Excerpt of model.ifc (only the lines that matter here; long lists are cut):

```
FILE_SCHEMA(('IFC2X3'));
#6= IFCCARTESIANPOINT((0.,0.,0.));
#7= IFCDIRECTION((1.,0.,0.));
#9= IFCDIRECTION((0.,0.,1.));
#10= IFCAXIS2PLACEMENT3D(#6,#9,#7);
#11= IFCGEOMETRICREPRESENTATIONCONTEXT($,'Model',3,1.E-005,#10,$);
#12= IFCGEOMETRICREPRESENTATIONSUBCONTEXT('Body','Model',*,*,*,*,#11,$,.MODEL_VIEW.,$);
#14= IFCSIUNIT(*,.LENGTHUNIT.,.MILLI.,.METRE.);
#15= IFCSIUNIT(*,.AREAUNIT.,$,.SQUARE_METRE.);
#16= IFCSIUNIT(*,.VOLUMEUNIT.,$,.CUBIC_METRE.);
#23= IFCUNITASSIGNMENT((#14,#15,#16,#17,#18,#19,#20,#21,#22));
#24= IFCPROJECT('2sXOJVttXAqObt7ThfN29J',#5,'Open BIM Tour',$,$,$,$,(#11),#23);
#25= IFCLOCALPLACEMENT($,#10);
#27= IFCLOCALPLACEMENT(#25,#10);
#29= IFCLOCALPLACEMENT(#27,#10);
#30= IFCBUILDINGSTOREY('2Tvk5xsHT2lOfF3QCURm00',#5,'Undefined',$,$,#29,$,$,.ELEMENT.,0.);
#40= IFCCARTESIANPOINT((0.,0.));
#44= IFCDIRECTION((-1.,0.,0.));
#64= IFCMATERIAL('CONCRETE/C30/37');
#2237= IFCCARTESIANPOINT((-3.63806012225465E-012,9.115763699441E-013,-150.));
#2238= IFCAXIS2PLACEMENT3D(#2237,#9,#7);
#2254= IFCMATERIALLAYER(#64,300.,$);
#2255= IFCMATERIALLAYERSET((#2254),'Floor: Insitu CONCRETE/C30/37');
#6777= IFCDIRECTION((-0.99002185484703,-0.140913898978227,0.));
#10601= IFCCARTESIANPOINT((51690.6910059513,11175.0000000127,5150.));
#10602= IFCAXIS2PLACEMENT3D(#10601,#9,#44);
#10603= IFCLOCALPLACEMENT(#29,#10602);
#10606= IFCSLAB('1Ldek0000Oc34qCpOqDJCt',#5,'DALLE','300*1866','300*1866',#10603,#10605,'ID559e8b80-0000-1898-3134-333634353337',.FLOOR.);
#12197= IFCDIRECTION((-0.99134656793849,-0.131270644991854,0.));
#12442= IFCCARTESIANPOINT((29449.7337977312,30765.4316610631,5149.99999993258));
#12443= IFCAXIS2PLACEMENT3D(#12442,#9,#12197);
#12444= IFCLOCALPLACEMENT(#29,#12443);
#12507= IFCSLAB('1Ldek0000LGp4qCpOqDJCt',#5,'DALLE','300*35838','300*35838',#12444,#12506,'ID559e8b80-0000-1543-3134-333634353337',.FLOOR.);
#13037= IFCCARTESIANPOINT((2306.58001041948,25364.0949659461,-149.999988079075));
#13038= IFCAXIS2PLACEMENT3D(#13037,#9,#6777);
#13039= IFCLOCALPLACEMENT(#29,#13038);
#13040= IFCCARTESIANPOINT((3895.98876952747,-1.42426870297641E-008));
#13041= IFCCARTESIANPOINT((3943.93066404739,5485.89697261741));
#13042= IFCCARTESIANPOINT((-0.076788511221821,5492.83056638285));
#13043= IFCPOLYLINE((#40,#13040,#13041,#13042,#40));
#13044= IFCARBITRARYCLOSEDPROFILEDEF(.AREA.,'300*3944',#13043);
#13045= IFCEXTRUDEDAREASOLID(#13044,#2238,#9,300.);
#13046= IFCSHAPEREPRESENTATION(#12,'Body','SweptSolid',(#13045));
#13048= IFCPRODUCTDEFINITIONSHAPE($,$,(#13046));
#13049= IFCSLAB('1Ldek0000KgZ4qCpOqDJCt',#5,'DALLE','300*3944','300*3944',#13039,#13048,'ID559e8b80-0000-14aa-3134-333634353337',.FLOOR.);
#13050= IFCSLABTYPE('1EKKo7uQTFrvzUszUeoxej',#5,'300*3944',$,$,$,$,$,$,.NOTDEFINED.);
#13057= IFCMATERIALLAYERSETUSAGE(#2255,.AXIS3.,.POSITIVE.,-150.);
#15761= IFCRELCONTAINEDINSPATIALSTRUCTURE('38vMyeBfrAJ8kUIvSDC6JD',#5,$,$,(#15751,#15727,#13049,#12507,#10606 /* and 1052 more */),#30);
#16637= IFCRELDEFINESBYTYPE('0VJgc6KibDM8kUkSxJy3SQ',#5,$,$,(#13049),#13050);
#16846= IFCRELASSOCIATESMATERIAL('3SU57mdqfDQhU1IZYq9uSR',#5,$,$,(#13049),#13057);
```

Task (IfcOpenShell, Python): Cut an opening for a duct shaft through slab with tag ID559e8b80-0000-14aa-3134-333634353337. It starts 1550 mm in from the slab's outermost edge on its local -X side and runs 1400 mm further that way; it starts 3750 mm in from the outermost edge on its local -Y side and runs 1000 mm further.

```python
import numpy as np
import ifcopenshell
import ifcopenshell.api.feature
import ifcopenshell.api.geometry
import ifcopenshell.api.root
import ifcopenshell.geom
import ifcopenshell.util.placement
import ifcopenshell.util.representation
import ifcopenshell.util.shape
import ifcopenshell.util.unit

model = ifcopenshell.open("model.ifc")
unit_scale = ifcopenshell.util.unit.calculate_unit_scale(model)
settings = ifcopenshell.geom.settings()


def volume(element):
    """Net volume in cubic metres, openings subtracted."""
    shape = ifcopenshell.geom.create_shape(settings, element)
    return ifcopenshell.util.shape.get_volume(shape.geometry)


slab = model.by_guid("1Ldek0000KgZ4qCpOqDJCt")
before = volume(slab)

# Extent in the slab's own axes, in metres. The edges named are its -X and -Y sides.
slab_shape = ifcopenshell.geom.create_shape(settings, slab)
vertices = ifcopenshell.util.shape.get_vertices(slab_shape.geometry)
x_min, y_min, bottom = vertices.min(axis=0)
top = vertices[:, 2].max()

opening = ifcopenshell.api.root.create_entity(model, ifc_class="IfcOpeningElement", name="Duct shaft opening")
context = ifcopenshell.util.representation.get_context(model, "Model", "Body", "MODEL_VIEW")
width, depth = 1.4, 1
outline = [(0.0, 0.0), (width, 0.0), (width, depth), (0.0, depth), (0.0, 0.0)]
# Overshoot both faces by 50 mm so the cut is clean.
shape = ifcopenshell.api.geometry.add_slab_representation(
    model, context=context, depth=top - bottom + 0.1, polyline=outline
)
ifcopenshell.api.geometry.assign_representation(model, product=opening, representation=shape)

matrix = ifcopenshell.util.placement.get_local_placement(slab.ObjectPlacement)
matrix[:, 3] = matrix @ np.append(np.array([x_min + 1.55, y_min + 3.75, bottom - 0.05]) / unit_scale, 1.0)
ifcopenshell.api.geometry.edit_object_placement(model, product=opening, matrix=matrix, is_si=False)
ifcopenshell.api.feature.add_feature(model, feature=opening, element=slab)

after = volume(slab)

print(f"slab volume {before:.3f} -> {after:.3f} m3")

model.write("model-out.ifc")
```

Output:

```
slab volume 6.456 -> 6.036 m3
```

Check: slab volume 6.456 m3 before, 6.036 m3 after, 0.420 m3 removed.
